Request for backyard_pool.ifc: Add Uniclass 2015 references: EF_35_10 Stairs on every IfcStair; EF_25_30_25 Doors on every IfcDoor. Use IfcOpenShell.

First a look at what the model holds.

```python
import ifcopenshell

model = ifcopenshell.open("backyard_pool.ifc")
print(model.schema)
print("classifications:", [c.Name for c in model.by_type("IfcClassification")])
for ifc_class in ("IfcDoor", "IfcRoof", "IfcStair", "IfcWall", "IfcWindow"):
    print(ifc_class, len(model.by_type(ifc_class)))
```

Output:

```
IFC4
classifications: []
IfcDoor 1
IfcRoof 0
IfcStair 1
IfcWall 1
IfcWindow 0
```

```python
import ifcopenshell
import ifcopenshell.api.classification

model = ifcopenshell.open("backyard_pool.ifc")

system = ifcopenshell.api.classification.add_classification(model, classification="Uniclass 2015")

codes = {
    "IfcStair": ("EF_35_10", "Stairs"),
    "IfcDoor": ("EF_25_30_25", "Doors"),
}
for ifc_class, (code, name) in codes.items():
    products = model.by_type(ifc_class)
    ifcopenshell.api.classification.add_reference(
        model, products=products, classification=system, identification=code, name=name
    )
    print(code, len(products))

model.write("backyard_pool_edited.ifc")
```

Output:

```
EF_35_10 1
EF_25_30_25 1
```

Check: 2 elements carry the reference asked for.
